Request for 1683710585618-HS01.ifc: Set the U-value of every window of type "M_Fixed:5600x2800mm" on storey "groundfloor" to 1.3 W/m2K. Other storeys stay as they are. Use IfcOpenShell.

First a look at what the model holds.

```python
import ifcopenshell
import ifcopenshell.util.element

model = ifcopenshell.open("1683710585618-HS01.ifc")
print(model.schema)
storey = next(s for s in model.by_type("IfcBuildingStorey") if s.Name == "groundfloor")
windows = [e for e in ifcopenshell.util.element.get_decomposition(storey) if e.is_a("IfcWindow")]
seen = {}
for e in windows:
    element_type = ifcopenshell.util.element.get_type(e)
    key = (element_type.Name if element_type != e and element_type else None, ifcopenshell.util.element.get_pset(e, "Pset_WindowCommon", "ThermalTransmittance"))
    seen[key] = seen.get(key, 0) + 1
for (name, value), count in sorted(seen.items(), key=str):
    print(count, "x", name, "|", value)
```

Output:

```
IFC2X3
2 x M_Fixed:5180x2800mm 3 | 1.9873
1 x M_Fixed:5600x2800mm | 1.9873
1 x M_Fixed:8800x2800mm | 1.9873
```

```python
import ifcopenshell
import ifcopenshell.api.pset
import ifcopenshell.util.element

model = ifcopenshell.open("1683710585618-HS01.ifc")

storey = next(s for s in model.by_type("IfcBuildingStorey") if s.Name == "groundfloor")
windows = [e for e in ifcopenshell.util.element.get_decomposition(storey) if e.is_a("IfcWindow")]

count = 0
for e in windows:
    element_type = ifcopenshell.util.element.get_type(e)
    if element_type in (None, e) or element_type.Name != "M_Fixed:5600x2800mm":
        continue
    # add_pset returns the element's existing set when there is one.
    pset = ifcopenshell.api.pset.add_pset(model, product=e, name="Pset_WindowCommon")
    ifcopenshell.api.pset.edit_pset(model, pset=pset, properties={"ThermalTransmittance": 1.3})
    count += 1

print(count, "windows updated")

model.write("1683710585618-HS01_edited.ifc")
```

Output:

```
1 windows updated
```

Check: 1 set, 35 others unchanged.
